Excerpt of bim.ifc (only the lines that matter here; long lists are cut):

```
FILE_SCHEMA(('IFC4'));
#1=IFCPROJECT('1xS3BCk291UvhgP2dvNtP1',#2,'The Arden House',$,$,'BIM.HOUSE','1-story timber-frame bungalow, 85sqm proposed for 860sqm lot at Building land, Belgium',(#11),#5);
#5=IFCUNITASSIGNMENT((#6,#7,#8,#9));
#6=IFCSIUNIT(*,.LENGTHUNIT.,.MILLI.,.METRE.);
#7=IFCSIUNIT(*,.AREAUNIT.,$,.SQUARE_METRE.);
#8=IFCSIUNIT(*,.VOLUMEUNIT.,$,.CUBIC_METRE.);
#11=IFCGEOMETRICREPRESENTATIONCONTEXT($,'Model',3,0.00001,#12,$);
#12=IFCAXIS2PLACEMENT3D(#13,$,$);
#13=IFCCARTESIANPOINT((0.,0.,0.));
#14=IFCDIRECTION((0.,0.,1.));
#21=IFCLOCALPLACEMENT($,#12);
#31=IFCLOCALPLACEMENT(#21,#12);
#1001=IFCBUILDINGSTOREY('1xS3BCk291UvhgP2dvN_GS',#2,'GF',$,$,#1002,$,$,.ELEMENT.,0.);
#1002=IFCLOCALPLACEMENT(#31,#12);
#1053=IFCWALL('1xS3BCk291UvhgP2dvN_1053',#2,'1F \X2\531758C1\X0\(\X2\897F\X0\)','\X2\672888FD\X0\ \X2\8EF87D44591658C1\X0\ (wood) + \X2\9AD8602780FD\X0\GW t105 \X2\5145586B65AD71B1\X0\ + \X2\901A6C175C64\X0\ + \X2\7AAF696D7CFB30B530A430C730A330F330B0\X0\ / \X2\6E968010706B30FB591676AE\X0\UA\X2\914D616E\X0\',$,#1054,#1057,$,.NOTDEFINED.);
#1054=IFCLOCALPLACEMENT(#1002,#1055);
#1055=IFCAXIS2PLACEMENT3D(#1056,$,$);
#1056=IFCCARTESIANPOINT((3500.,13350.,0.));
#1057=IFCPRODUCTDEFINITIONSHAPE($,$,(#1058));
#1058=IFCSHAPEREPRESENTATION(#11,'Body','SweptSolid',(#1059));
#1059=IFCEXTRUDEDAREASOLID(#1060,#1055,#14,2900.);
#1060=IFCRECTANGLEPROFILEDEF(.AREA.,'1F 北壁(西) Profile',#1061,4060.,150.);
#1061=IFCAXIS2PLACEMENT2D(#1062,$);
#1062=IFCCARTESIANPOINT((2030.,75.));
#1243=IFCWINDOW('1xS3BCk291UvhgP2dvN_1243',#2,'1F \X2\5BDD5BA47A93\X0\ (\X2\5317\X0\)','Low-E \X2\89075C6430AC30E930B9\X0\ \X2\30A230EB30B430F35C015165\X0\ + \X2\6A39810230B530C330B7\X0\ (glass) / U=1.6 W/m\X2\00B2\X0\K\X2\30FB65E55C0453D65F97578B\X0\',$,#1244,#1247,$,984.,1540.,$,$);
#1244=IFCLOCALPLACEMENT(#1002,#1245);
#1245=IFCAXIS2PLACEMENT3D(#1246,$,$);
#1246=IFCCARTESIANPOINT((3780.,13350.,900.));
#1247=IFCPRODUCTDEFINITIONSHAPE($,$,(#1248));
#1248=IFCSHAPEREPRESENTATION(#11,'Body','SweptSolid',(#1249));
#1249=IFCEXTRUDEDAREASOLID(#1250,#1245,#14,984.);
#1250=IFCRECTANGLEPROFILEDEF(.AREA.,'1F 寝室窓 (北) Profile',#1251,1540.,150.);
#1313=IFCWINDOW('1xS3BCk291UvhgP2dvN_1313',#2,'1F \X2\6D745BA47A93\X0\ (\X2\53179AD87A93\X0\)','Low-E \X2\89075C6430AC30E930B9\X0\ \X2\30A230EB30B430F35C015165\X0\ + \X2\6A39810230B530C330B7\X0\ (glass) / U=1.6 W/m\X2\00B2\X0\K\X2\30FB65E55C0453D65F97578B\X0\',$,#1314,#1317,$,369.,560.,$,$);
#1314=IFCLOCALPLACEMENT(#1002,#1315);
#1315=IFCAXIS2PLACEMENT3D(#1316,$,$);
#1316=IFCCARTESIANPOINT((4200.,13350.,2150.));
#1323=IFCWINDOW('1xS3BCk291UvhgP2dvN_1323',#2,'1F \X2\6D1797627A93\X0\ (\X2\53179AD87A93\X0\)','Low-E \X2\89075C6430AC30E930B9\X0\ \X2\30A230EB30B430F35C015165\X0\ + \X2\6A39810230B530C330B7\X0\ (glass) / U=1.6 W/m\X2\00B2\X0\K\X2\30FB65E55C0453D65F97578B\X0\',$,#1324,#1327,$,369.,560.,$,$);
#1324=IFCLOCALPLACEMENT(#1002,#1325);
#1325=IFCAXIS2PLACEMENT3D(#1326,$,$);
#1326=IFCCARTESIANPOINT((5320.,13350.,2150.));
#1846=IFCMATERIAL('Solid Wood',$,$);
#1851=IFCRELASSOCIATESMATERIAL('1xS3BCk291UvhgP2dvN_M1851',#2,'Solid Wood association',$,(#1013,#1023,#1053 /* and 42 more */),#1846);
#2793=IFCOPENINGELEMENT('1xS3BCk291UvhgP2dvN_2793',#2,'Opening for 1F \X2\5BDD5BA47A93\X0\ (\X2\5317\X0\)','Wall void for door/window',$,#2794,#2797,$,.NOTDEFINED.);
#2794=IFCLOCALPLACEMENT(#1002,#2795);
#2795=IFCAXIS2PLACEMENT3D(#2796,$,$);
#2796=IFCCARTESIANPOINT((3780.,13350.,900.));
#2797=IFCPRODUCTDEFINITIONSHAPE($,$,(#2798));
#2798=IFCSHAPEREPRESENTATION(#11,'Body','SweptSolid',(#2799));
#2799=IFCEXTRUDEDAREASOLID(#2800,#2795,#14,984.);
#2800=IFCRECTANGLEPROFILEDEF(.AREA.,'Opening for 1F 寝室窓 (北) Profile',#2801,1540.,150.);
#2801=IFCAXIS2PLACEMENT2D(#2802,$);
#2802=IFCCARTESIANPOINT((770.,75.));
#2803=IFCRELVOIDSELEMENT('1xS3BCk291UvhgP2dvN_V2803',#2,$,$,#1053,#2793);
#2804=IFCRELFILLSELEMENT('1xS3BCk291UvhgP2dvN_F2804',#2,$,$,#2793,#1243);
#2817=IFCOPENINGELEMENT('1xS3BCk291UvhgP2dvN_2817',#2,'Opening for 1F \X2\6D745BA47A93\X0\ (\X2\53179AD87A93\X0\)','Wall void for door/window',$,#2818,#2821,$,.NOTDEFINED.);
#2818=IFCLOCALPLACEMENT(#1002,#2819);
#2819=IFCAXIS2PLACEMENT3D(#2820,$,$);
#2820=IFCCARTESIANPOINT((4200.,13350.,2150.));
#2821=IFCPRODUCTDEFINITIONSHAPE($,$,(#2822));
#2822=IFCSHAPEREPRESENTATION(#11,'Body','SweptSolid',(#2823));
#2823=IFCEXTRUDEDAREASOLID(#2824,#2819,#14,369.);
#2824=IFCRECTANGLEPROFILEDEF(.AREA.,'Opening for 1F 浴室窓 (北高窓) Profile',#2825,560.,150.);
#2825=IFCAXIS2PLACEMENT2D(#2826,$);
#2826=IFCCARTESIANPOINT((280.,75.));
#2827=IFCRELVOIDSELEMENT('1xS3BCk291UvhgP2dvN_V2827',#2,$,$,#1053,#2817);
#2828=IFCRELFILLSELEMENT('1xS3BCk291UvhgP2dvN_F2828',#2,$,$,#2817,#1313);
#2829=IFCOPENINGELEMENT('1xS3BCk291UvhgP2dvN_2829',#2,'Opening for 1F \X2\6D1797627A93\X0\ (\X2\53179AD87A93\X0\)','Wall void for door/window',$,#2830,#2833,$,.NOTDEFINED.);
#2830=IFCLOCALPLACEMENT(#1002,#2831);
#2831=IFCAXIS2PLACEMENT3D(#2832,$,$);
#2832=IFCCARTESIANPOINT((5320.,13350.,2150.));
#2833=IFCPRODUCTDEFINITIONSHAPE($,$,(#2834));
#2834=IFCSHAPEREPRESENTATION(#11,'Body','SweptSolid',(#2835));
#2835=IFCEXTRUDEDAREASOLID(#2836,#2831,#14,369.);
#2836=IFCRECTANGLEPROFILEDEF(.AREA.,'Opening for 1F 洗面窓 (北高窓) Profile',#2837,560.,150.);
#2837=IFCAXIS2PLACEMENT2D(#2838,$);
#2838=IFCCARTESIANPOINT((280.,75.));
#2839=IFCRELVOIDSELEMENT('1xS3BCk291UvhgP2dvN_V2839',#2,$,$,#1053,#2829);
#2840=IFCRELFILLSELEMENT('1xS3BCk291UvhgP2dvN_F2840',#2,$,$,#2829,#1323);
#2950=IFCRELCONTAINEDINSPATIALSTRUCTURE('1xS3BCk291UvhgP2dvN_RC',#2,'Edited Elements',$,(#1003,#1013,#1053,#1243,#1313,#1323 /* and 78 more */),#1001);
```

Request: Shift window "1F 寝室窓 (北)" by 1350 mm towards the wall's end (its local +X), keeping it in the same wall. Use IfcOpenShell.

```python
import ifcopenshell
import ifcopenshell.api.geometry
import ifcopenshell.util.placement

model = ifcopenshell.open("bim.ifc")

window = model.by_id(1243)
opening = window.FillsVoids[0].RelatingOpeningElement
wall = opening.VoidsElements[0].RelatingBuildingElement

wall_matrix = ifcopenshell.util.placement.get_local_placement(wall.ObjectPlacement)
shift = wall_matrix[:3, 0] * 1350.0
before = ifcopenshell.util.placement.get_local_placement(window.ObjectPlacement)[:3, 3].copy()

# The window is not placed relative to its opening, so move both.
for product in (opening, window):
    matrix = ifcopenshell.util.placement.get_local_placement(product.ObjectPlacement)
    matrix[:3, 3] += shift
    ifcopenshell.api.geometry.edit_object_placement(model, product=product, matrix=matrix, is_si=False)

after = ifcopenshell.util.placement.get_local_placement(window.ObjectPlacement)[:3, 3]
print("window moved by", (after - before).round(3) + 0.0)

model.write("bim_rev.ifc")
```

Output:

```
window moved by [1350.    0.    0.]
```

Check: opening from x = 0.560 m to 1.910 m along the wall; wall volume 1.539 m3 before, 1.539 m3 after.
